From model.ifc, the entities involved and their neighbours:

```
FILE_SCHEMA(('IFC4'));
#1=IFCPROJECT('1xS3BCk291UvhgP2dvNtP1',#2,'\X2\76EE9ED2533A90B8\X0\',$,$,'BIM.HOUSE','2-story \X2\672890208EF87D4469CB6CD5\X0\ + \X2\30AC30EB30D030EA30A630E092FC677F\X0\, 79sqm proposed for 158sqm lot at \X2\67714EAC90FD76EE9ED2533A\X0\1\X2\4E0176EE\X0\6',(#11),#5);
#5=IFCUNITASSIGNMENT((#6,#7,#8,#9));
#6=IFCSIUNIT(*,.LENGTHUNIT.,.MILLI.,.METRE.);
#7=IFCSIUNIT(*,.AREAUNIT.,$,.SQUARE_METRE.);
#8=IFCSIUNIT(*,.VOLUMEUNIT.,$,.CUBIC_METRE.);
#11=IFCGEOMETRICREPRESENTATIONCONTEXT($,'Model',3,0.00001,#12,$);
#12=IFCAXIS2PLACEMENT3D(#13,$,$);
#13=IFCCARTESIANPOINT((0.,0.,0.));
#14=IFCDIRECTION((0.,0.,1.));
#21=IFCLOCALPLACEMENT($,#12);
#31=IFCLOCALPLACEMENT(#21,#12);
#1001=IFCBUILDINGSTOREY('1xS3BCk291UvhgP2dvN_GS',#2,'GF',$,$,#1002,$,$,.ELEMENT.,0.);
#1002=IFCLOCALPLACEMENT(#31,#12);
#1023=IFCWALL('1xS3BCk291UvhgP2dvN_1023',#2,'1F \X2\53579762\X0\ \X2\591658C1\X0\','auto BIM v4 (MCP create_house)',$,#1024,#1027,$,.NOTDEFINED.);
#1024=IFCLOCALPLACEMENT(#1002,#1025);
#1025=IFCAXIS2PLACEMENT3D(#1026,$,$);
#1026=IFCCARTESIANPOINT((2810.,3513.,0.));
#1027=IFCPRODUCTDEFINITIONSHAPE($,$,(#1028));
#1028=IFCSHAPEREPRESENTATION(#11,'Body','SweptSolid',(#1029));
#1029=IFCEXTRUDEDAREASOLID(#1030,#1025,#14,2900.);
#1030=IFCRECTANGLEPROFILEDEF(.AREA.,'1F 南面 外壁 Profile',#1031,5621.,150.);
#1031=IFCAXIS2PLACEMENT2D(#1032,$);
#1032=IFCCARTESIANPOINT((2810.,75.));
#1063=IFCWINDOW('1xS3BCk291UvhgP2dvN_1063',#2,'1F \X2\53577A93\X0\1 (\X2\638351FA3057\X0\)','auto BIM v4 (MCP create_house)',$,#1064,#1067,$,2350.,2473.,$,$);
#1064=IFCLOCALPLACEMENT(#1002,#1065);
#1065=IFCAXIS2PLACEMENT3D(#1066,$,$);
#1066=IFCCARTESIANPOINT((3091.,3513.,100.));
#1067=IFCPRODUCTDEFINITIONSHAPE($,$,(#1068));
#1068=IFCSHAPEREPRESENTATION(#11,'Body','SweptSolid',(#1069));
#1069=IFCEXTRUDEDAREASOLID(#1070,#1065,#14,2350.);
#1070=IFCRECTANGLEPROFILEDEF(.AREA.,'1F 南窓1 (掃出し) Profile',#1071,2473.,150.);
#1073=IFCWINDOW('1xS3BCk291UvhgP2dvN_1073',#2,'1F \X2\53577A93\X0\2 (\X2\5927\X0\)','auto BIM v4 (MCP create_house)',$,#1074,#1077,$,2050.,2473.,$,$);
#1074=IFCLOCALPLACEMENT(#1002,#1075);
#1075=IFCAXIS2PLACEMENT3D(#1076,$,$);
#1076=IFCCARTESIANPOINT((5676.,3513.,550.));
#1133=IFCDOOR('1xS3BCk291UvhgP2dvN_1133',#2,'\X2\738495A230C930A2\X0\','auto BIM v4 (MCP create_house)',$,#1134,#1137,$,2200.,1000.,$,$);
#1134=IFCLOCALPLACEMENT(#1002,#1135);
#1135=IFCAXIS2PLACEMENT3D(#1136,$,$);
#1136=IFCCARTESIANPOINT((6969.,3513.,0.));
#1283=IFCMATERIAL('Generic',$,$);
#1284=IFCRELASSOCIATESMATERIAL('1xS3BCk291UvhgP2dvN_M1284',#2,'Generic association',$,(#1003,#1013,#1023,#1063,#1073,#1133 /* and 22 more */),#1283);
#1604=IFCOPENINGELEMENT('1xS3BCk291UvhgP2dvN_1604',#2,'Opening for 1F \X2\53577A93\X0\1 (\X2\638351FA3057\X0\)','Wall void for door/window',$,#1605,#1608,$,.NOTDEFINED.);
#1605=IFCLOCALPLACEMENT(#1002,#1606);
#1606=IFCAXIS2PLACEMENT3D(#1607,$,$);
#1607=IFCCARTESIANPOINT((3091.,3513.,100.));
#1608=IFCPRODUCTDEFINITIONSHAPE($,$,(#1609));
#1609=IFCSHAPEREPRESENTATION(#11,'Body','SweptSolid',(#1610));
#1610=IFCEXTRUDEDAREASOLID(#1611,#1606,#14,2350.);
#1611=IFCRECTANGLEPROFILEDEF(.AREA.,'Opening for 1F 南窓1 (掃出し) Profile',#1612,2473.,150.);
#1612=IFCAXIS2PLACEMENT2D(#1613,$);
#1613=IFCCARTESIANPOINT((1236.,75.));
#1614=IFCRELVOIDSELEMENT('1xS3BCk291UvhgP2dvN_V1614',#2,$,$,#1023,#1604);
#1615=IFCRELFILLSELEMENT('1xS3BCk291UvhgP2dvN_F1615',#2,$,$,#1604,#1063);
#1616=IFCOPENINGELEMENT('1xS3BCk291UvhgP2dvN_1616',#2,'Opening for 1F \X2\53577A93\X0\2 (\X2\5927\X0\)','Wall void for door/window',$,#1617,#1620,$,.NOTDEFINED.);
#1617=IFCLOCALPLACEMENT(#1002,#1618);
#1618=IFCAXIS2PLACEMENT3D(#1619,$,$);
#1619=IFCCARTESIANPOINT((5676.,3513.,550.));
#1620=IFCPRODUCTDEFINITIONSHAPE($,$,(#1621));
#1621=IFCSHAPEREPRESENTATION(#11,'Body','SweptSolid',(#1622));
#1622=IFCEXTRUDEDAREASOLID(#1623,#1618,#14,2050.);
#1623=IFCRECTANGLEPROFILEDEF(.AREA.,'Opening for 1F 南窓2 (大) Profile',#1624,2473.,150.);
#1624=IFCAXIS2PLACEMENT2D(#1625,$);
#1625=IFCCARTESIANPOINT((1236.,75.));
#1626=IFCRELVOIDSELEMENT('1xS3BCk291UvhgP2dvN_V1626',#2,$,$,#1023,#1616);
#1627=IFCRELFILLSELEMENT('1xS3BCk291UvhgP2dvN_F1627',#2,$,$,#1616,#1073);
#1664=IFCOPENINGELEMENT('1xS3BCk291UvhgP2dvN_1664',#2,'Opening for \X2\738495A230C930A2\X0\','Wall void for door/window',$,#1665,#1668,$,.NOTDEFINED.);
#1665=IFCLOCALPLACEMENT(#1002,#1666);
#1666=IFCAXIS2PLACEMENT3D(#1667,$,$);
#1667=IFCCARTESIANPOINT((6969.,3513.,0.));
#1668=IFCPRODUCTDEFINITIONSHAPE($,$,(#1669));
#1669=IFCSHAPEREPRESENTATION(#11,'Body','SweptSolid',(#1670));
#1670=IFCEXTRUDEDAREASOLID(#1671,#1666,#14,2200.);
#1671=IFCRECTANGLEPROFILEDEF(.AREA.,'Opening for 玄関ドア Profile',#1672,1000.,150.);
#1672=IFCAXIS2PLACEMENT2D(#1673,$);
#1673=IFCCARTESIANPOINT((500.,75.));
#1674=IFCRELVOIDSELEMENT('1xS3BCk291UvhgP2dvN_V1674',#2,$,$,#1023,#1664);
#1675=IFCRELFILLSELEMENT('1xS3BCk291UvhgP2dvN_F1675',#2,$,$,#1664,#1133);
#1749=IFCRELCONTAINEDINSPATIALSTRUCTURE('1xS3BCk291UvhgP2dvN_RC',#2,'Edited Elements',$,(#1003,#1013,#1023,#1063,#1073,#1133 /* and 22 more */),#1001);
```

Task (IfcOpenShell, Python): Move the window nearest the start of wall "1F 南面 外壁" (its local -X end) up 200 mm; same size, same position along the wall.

```python
import numpy as np
import ifcopenshell
import ifcopenshell.api.geometry
import ifcopenshell.util.placement
import ifcopenshell.util.unit

model = ifcopenshell.open("model.ifc")
unit_scale = ifcopenshell.util.unit.calculate_unit_scale(model)

window = model.by_guid("1xS3BCk291UvhgP2dvN_1063")
opening = window.FillsVoids[0].RelatingOpeningElement
dz = 200.0

shift = np.array([0.0, 0.0, dz])
# The window is not placed relative to its opening, so move both.
for product in (opening, window):
    matrix = ifcopenshell.util.placement.get_local_placement(product.ObjectPlacement)
    matrix[:3, 3] += shift
    ifcopenshell.api.geometry.edit_object_placement(model, product=product, matrix=matrix, is_si=False)

print(f"moved by {dz * unit_scale:+.3f} m")

model.write("model_edited.ifc")
```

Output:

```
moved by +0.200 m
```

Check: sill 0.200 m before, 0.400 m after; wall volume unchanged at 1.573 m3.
